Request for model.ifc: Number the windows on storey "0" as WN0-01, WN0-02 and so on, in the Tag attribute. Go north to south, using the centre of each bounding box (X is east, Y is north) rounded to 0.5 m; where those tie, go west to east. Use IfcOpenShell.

First a look at what the model holds.

```python
import ifcopenshell
import ifcopenshell.util.element
import ifcopenshell.util.placement

model = ifcopenshell.open("model.ifc")
print(model.schema)
storey = next(s for s in model.by_type("IfcBuildingStorey") if s.Name == "0")
windows = [e for e in ifcopenshell.util.element.get_decomposition(storey) if e.is_a("IfcWindow")]
for e in sorted(windows, key=lambda e: e.id()):
    origin = ifcopenshell.util.placement.get_local_placement(e.ObjectPlacement)[:3, 3]
    print(e.id(), e.Tag, e.Name, origin.round(2) + 0.0, sep=" | ")
```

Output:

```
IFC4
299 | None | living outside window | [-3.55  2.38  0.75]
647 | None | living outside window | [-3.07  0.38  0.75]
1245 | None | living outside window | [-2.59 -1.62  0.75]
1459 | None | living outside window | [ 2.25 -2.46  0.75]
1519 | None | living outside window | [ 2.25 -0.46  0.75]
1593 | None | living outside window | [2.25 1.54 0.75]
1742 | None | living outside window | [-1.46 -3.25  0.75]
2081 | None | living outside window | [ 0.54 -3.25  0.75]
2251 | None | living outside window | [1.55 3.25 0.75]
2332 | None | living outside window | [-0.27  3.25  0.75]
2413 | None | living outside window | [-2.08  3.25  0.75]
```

```python
import ifcopenshell
import ifcopenshell.geom
import ifcopenshell.util.element
import ifcopenshell.util.shape

model = ifcopenshell.open("model.ifc")
settings = ifcopenshell.geom.settings()
settings.set("use-world-coords", True)


def centre(element):
    shape = ifcopenshell.geom.create_shape(settings, element)
    return ifcopenshell.util.shape.get_bbox_centroid(shape.geometry)


storey = next(s for s in model.by_type("IfcBuildingStorey") if s.Name == "0")
windows = [e for e in ifcopenshell.util.element.get_decomposition(storey) if e.is_a("IfcWindow")]

# Insertion points can sit at a corner or the storey origin, so sort by the geometry (in metres).
centres = {e: centre(e) for e in windows}
windows.sort(key=lambda e: (-round(centres[e][1] / 0.5), centres[e][0]))

for i, e in enumerate(windows, start=1):
    number = f"WN0-{i:02d}"
    e.Tag = number
    print(e.id(), number)

model.write("model_edited.ifc")
```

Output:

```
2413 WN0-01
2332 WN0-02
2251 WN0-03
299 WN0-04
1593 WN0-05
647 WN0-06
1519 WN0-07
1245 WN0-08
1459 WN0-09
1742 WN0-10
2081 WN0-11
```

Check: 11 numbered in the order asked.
